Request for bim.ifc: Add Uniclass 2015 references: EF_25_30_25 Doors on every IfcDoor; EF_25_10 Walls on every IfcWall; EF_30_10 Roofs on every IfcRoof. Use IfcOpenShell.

First a look at what the model holds.

```python
import ifcopenshell

model = ifcopenshell.open("bim.ifc")
print(model.schema)
print("classifications:", [c.Name for c in model.by_type("IfcClassification")])
for ifc_class in ("IfcDoor", "IfcRoof", "IfcStair", "IfcWall", "IfcWindow"):
    print(ifc_class, len(model.by_type(ifc_class)))
```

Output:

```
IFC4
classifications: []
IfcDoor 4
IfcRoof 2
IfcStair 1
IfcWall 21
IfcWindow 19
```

```python
import ifcopenshell
import ifcopenshell.api.classification

model = ifcopenshell.open("bim.ifc")

system = ifcopenshell.api.classification.add_classification(model, classification="Uniclass 2015")

codes = {
    "IfcDoor": ("EF_25_30_25", "Doors"),
    "IfcWall": ("EF_25_10", "Walls"),
    "IfcRoof": ("EF_30_10", "Roofs"),
}
for ifc_class, (code, name) in codes.items():
    products = model.by_type(ifc_class)
    ifcopenshell.api.classification.add_reference(
        model, products=products, classification=system, identification=code, name=name
    )
    print(code, len(products))

model.write("bim-out.ifc")
```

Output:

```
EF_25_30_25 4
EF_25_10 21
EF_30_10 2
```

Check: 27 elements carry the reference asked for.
